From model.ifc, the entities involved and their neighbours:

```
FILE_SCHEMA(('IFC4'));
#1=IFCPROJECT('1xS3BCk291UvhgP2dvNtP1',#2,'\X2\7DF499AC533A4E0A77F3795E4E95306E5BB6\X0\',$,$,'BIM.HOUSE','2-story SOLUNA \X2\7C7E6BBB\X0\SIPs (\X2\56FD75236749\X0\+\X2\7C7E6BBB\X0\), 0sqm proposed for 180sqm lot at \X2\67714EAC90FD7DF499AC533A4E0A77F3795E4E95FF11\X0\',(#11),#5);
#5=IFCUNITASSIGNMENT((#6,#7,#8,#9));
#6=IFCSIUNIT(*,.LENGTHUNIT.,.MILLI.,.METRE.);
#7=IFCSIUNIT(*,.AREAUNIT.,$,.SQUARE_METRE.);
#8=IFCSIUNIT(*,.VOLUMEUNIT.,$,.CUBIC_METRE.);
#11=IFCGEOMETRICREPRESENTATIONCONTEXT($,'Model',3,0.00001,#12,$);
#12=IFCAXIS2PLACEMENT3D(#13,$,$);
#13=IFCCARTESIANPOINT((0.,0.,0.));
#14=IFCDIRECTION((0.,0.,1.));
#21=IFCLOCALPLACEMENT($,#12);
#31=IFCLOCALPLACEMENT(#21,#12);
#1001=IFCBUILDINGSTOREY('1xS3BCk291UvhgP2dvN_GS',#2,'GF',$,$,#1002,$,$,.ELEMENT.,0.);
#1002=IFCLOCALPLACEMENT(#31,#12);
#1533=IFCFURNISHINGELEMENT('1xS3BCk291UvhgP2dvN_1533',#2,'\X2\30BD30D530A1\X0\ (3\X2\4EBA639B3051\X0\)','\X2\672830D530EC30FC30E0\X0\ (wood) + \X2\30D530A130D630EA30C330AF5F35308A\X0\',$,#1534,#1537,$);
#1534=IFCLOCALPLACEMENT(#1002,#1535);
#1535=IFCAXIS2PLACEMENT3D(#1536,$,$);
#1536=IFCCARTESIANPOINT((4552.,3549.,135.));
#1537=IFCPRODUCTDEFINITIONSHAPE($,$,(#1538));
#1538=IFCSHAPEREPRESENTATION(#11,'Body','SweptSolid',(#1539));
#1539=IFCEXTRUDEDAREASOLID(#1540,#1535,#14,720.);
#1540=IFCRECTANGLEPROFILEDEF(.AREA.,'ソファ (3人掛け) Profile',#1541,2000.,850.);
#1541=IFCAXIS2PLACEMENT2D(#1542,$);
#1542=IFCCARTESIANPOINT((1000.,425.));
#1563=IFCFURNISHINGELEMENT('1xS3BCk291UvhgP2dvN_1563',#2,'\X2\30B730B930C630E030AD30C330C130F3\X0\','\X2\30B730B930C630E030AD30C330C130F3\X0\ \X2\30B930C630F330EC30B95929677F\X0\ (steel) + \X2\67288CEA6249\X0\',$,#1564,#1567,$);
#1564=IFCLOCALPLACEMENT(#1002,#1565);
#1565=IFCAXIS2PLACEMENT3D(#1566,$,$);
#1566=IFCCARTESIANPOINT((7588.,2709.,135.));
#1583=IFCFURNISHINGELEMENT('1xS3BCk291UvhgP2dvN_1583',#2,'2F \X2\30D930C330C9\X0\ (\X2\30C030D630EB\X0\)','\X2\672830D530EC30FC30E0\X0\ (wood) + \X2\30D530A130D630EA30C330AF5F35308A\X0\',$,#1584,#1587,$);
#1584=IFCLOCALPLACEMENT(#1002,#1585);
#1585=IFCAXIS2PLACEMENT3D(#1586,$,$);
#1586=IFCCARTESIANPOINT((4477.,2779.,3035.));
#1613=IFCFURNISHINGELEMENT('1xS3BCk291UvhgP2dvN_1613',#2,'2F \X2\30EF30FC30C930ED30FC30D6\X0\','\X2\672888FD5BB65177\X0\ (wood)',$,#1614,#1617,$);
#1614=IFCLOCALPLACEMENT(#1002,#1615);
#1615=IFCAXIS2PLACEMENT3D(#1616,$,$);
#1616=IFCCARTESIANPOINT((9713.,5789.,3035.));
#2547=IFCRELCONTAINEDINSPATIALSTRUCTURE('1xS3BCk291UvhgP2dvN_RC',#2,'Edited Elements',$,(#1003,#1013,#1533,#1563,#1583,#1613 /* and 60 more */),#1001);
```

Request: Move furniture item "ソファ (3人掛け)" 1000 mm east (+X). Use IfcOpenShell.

```python
import ifcopenshell
import ifcopenshell.api.geometry
import ifcopenshell.util.placement

model = ifcopenshell.open("model.ifc")

item = model.by_guid("1xS3BCk291UvhgP2dvN_1533")
matrix = ifcopenshell.util.placement.get_local_placement(item.ObjectPlacement)
matrix[0, 3] += 1000.0
ifcopenshell.api.geometry.edit_object_placement(model, product=item, matrix=matrix, is_si=False)

print(ifcopenshell.util.placement.get_local_placement(item.ObjectPlacement).round(3) + 0.0)

model.write("model-out.ifc")
```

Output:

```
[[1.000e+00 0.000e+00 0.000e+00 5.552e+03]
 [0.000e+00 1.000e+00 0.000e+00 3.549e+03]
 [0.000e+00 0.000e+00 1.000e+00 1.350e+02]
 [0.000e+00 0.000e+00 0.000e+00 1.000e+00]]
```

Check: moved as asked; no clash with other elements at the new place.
